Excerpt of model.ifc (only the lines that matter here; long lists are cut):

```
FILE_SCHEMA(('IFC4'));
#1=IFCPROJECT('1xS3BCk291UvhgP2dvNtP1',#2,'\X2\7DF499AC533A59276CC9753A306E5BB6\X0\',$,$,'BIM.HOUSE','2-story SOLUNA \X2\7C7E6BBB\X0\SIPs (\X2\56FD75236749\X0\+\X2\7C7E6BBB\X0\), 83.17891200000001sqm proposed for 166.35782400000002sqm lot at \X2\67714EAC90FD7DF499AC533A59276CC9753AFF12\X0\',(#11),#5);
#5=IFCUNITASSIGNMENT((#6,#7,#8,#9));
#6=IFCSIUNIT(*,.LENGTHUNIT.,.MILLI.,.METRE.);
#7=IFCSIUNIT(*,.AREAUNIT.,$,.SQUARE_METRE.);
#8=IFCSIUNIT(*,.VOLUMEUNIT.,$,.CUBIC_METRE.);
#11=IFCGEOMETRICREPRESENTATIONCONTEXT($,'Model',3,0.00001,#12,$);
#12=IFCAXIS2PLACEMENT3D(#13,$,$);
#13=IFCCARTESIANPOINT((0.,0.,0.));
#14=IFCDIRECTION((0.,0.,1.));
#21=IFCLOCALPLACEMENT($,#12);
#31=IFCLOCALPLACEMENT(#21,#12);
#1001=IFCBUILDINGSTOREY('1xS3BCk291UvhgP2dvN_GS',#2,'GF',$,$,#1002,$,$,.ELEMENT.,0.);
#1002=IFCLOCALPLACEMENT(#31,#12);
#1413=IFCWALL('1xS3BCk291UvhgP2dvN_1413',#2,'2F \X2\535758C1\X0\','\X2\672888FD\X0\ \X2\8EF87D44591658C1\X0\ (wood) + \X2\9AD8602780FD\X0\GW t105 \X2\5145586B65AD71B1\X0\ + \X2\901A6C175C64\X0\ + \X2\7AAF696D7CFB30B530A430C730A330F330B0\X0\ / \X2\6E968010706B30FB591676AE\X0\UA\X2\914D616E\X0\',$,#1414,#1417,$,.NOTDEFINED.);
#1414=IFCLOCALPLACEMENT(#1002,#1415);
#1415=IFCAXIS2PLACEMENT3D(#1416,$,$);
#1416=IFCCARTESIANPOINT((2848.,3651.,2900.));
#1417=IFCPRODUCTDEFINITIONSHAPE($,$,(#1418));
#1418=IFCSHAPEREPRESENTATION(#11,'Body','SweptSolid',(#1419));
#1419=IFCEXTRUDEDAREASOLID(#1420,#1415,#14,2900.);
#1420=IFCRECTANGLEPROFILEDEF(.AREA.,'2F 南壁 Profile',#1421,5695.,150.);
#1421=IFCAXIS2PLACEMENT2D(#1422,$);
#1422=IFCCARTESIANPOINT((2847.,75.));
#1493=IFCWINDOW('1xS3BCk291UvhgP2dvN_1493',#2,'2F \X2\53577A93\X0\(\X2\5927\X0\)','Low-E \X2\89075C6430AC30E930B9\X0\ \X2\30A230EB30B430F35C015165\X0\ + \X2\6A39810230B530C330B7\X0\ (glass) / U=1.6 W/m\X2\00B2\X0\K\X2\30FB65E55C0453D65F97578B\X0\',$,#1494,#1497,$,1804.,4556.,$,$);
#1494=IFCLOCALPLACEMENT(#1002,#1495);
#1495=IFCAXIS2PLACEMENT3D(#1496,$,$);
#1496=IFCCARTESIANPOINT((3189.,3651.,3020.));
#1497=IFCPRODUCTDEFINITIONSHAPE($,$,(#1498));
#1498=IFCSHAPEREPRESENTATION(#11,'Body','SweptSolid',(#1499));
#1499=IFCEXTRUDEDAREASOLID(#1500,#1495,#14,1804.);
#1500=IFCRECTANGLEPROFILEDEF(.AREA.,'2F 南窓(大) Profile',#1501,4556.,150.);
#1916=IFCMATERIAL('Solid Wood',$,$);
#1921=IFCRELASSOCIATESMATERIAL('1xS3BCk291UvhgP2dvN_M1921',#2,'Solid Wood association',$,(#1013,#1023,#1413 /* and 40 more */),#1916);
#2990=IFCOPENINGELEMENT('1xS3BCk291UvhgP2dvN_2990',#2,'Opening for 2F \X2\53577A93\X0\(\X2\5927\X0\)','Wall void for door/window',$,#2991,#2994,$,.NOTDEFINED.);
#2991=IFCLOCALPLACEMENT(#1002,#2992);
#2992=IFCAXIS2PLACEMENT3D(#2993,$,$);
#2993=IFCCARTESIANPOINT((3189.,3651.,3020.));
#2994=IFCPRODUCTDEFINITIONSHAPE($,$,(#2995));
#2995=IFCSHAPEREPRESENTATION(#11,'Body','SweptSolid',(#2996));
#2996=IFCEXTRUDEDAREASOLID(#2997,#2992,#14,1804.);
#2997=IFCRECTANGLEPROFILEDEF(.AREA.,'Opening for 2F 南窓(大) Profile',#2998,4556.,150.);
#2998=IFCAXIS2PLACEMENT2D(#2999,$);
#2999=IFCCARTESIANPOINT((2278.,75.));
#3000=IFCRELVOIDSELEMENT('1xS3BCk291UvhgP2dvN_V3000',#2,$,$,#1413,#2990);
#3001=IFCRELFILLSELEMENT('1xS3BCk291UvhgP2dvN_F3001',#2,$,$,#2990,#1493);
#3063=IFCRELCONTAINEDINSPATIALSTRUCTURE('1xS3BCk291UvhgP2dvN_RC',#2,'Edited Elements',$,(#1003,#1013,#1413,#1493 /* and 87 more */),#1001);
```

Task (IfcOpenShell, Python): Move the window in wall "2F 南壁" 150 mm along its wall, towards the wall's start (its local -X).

```python
import ifcopenshell
import ifcopenshell.api.geometry
import ifcopenshell.util.placement
import ifcopenshell.util.unit

model = ifcopenshell.open("model.ifc")
unit_scale = ifcopenshell.util.unit.calculate_unit_scale(model)

window = model.by_guid("1xS3BCk291UvhgP2dvN_1493")
opening = window.FillsVoids[0].RelatingOpeningElement
wall = opening.VoidsElements[0].RelatingBuildingElement

wall_matrix = ifcopenshell.util.placement.get_local_placement(wall.ObjectPlacement)
shift = wall_matrix[:3, 0] * -0.15 / unit_scale
before = ifcopenshell.util.placement.get_local_placement(window.ObjectPlacement)[:3, 3].copy()

# The window is not placed relative to its opening, so move both.
for product in (opening, window):
    matrix = ifcopenshell.util.placement.get_local_placement(product.ObjectPlacement)
    matrix[:3, 3] += shift
    ifcopenshell.api.geometry.edit_object_placement(model, product=product, matrix=matrix, is_si=False)

after = ifcopenshell.util.placement.get_local_placement(window.ObjectPlacement)[:3, 3]
print("window moved by", (after - before).round(3) + 0.0)

model.write("model_rev.ifc")
```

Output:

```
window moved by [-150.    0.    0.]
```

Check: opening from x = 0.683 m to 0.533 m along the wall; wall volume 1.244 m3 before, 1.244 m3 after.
